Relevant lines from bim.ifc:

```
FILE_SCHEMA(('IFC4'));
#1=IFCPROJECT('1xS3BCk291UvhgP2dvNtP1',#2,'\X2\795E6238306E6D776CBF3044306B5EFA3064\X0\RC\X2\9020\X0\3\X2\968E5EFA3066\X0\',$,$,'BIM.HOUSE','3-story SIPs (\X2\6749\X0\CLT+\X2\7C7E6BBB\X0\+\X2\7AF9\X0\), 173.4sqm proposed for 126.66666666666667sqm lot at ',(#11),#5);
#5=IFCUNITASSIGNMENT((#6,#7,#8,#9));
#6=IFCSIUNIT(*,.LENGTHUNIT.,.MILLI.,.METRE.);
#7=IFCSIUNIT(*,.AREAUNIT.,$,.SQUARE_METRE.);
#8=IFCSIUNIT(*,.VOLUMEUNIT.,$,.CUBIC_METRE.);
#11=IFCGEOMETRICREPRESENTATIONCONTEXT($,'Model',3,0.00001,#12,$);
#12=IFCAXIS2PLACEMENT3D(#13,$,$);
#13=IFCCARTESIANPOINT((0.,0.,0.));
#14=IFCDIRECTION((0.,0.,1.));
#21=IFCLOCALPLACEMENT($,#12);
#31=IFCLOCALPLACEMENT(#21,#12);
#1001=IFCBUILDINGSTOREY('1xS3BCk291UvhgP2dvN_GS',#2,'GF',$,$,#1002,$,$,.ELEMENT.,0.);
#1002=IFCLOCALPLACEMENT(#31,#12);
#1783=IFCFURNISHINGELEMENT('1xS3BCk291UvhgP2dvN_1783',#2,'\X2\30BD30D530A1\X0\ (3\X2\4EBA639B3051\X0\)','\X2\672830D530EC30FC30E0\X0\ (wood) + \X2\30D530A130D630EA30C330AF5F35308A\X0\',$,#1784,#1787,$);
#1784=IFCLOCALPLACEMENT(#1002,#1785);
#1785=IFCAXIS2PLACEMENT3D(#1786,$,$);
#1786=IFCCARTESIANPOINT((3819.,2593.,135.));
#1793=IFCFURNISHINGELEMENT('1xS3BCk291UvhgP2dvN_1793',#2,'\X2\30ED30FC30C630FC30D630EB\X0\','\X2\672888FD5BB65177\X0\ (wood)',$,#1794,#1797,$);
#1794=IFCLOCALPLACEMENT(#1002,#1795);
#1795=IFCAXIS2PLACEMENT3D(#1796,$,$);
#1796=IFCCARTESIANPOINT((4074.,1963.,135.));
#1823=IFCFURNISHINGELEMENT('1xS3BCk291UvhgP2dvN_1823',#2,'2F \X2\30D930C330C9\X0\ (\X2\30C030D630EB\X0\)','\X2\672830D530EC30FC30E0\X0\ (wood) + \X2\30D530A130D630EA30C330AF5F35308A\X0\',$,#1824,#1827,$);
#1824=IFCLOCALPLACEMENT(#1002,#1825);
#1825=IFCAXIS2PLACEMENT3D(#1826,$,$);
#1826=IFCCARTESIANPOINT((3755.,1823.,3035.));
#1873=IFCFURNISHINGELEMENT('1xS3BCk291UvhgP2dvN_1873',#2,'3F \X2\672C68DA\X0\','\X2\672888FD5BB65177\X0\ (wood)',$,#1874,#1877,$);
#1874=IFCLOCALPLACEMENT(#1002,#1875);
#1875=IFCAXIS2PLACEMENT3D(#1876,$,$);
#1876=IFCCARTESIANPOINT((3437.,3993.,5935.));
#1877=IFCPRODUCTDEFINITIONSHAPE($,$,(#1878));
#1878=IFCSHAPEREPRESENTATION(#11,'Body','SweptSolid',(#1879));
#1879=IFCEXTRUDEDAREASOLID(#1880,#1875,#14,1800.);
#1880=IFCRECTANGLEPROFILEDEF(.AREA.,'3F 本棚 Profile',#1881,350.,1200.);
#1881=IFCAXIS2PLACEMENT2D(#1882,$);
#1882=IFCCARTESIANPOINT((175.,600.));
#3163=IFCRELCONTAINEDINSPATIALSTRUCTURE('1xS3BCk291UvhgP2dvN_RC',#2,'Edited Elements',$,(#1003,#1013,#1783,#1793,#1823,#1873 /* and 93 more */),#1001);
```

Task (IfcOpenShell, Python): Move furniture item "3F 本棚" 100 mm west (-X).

```python
import ifcopenshell
import ifcopenshell.api.geometry
import ifcopenshell.util.placement

model = ifcopenshell.open("bim.ifc")

item = model.by_guid("1xS3BCk291UvhgP2dvN_1873")
matrix = ifcopenshell.util.placement.get_local_placement(item.ObjectPlacement)
matrix[0, 3] -= 100.0
ifcopenshell.api.geometry.edit_object_placement(model, product=item, matrix=matrix, is_si=False)

print(ifcopenshell.util.placement.get_local_placement(item.ObjectPlacement).round(3) + 0.0)

model.write("bim_rev.ifc")
```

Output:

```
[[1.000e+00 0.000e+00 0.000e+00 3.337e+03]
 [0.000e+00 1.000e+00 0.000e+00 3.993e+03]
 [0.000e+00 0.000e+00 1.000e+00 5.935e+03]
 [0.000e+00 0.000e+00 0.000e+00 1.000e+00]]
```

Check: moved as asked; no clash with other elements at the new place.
